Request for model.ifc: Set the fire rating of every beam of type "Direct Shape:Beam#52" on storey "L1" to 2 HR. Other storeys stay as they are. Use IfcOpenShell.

First a look at what the model holds.

```python
import ifcopenshell
import ifcopenshell.util.element

model = ifcopenshell.open("model.ifc")
print(model.schema)
storey = next(s for s in model.by_type("IfcBuildingStorey") if s.Name == "L1")
beams = [e for e in ifcopenshell.util.element.get_decomposition(storey) if e.is_a("IfcBeam")]
seen = {}
for e in beams:
    element_type = ifcopenshell.util.element.get_type(e)
    key = (element_type.Name if element_type != e and element_type else None, ifcopenshell.util.element.get_pset(e, "Pset_BeamCommon", "FireRating"))
    seen[key] = seen.get(key, 0) + 1
for (name, value), count in sorted(seen.items(), key=str):
    print(count, "x", name, "|", value)
```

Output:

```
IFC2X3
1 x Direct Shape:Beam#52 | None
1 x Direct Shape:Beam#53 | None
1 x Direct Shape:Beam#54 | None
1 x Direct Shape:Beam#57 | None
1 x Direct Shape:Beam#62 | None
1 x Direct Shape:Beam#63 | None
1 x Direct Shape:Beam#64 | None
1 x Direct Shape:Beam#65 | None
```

```python
import ifcopenshell
import ifcopenshell.api.pset
import ifcopenshell.util.element

model = ifcopenshell.open("model.ifc")

storey = next(s for s in model.by_type("IfcBuildingStorey") if s.Name == "L1")
beams = [e for e in ifcopenshell.util.element.get_decomposition(storey) if e.is_a("IfcBeam")]

count = 0
for e in beams:
    element_type = ifcopenshell.util.element.get_type(e)
    if element_type in (None, e) or element_type.Name != "Direct Shape:Beam#52":
        continue
    # add_pset returns the element's existing set when there is one.
    pset = ifcopenshell.api.pset.add_pset(model, product=e, name="Pset_BeamCommon")
    ifcopenshell.api.pset.edit_pset(model, pset=pset, properties={"FireRating": "2 HR"})
    count += 1

print(count, "beams updated")

model.write("model_edited.ifc")
```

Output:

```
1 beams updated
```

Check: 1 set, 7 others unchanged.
